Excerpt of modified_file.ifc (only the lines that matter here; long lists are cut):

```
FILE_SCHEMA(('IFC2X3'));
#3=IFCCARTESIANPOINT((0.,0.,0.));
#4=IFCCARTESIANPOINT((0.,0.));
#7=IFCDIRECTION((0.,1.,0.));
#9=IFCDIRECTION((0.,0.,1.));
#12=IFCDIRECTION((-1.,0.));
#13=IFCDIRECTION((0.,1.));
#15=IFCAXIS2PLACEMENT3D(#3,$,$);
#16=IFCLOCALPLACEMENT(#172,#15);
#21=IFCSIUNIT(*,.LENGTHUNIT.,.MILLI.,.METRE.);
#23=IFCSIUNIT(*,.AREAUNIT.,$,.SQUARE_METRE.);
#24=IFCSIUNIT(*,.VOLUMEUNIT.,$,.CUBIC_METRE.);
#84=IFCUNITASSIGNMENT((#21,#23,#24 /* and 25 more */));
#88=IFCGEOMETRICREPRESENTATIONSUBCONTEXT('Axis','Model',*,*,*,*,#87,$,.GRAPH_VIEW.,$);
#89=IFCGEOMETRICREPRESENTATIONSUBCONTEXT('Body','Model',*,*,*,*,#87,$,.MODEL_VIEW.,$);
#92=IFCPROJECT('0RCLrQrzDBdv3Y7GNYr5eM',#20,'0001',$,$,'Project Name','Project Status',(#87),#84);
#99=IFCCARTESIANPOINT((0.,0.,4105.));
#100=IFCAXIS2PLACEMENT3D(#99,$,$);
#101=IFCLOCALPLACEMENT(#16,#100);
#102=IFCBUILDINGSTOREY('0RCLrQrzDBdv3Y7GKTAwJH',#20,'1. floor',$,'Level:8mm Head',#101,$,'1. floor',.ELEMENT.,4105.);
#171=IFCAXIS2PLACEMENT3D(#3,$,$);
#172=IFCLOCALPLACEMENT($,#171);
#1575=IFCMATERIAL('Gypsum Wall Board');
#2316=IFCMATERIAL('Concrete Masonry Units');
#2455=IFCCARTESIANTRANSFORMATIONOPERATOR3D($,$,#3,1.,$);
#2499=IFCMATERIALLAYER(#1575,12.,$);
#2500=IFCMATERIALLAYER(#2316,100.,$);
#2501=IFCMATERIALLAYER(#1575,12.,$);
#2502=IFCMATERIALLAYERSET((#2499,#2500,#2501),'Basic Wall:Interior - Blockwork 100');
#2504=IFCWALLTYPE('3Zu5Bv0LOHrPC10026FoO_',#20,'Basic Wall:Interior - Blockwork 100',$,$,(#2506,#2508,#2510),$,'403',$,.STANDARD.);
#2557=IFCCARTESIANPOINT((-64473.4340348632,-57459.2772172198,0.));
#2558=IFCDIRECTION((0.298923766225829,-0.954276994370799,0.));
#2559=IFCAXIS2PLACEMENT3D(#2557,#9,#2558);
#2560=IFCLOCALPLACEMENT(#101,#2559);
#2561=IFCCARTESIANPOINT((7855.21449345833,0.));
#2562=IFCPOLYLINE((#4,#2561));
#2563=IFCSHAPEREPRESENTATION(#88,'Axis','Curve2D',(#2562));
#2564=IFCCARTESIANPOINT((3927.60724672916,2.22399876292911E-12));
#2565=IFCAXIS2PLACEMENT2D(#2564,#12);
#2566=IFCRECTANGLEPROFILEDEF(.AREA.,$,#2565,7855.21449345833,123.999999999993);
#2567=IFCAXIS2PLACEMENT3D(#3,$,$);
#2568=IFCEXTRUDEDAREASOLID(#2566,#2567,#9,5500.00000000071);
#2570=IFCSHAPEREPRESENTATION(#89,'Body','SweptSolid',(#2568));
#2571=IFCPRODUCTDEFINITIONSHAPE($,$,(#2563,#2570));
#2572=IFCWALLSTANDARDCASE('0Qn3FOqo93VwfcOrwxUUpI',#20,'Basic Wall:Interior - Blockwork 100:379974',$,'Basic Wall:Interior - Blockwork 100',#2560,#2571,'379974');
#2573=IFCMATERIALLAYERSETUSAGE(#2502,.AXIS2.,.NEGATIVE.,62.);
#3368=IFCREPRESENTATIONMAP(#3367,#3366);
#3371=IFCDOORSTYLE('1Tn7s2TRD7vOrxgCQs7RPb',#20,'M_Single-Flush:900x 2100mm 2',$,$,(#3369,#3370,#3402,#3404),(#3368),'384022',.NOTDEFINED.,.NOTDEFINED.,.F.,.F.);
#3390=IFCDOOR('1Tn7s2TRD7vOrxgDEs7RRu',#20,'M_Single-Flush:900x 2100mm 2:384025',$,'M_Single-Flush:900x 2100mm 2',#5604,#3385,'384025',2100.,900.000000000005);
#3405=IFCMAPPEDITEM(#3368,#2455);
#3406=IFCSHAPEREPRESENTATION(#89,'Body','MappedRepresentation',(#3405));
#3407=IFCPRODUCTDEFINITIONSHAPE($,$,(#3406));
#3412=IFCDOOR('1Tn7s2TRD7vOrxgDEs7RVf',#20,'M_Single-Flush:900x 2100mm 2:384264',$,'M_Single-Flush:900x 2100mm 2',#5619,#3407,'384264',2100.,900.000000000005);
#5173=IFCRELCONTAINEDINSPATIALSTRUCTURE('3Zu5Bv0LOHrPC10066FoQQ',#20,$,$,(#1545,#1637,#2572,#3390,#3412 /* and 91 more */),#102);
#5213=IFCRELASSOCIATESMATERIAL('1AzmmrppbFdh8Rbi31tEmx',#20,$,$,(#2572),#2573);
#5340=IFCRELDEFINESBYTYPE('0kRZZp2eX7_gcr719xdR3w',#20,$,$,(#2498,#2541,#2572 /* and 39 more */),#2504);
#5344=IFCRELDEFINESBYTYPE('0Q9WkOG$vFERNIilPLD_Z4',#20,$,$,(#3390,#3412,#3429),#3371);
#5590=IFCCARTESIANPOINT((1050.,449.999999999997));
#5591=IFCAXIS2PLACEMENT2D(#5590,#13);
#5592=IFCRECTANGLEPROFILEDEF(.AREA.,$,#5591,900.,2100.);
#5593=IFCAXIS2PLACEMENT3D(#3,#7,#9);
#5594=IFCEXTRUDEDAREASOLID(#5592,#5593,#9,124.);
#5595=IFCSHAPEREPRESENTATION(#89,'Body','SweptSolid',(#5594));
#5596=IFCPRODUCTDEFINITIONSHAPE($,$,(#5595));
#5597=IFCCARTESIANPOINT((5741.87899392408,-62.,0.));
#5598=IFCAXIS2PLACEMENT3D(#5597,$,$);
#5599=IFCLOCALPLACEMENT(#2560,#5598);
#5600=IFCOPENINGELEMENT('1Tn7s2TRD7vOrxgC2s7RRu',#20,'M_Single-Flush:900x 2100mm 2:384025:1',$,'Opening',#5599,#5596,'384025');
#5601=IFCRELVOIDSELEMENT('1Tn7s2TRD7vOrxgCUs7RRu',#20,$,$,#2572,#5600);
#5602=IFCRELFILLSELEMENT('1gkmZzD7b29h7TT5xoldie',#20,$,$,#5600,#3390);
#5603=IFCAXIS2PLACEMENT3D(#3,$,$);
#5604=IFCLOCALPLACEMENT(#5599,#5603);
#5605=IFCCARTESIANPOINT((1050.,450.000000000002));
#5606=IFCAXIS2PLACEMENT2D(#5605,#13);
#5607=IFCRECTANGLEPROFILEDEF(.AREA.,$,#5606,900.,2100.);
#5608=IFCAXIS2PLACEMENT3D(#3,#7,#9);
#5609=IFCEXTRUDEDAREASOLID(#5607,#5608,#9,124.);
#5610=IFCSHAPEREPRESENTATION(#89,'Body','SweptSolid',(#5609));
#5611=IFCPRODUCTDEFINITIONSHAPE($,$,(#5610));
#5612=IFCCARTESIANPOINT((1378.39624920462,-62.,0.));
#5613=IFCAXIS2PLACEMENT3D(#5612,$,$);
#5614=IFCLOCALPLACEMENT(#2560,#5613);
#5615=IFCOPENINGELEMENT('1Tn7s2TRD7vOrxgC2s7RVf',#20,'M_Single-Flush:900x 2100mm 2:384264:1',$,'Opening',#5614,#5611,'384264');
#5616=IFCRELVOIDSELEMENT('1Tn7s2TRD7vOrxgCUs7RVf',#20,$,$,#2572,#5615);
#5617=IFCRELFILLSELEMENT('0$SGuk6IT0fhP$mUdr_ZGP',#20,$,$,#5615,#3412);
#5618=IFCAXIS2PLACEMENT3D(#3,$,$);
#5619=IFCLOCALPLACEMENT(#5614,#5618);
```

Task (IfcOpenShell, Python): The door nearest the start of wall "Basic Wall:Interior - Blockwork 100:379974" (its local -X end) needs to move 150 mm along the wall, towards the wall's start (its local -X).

```python
import ifcopenshell
import ifcopenshell.api.geometry
import ifcopenshell.util.placement

model = ifcopenshell.open("modified_file.ifc")

door = model.by_guid("1Tn7s2TRD7vOrxgDEs7RVf")
opening = door.FillsVoids[0].RelatingOpeningElement
wall = opening.VoidsElements[0].RelatingBuildingElement

wall_matrix = ifcopenshell.util.placement.get_local_placement(wall.ObjectPlacement)
shift = wall_matrix[:3, 0] * -150.0
before = ifcopenshell.util.placement.get_local_placement(door.ObjectPlacement)[:3, 3].copy()

# The door is placed relative to its opening, so it follows when the opening moves.
matrix = ifcopenshell.util.placement.get_local_placement(opening.ObjectPlacement)
matrix[:3, 3] += shift
ifcopenshell.api.geometry.edit_object_placement(
    model, product=opening, matrix=matrix, is_si=False, should_transform_children=True
)

after = ifcopenshell.util.placement.get_local_placement(door.ObjectPlacement)[:3, 3]
print("door moved by", (after - before).round(3) + 0.0)

model.write("modified_file_rev.ifc")
```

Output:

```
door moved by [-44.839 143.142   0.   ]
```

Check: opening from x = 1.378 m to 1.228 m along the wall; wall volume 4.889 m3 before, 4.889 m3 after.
